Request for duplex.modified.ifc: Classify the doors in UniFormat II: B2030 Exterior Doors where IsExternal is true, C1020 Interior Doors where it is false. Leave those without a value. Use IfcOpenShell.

First a look at what the model holds.

```python
import ifcopenshell
import ifcopenshell.util.element

model = ifcopenshell.open("duplex.modified.ifc")
print(model.schema)
print("classifications:", [c.Name for c in model.by_type("IfcClassification")])
values = [ifcopenshell.util.element.get_pset(e, "Pset_DoorCommon", "IsExternal") for e in model.by_type("IfcDoor")]
for value in (True, False, None):
    print("IsExternal", value, values.count(value))
```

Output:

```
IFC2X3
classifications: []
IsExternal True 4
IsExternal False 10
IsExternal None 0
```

```python
import ifcopenshell
import ifcopenshell.api.classification
import ifcopenshell.util.element

model = ifcopenshell.open("duplex.modified.ifc")

# IFC2X3 requires Source and Edition and has no link from the project to the system.
system = model.create_entity("IfcClassification", Source="ASTM", Edition="E1557", Name="UniFormat II")

doors = model.by_type("IfcDoor")
external = {e: ifcopenshell.util.element.get_pset(e, "Pset_DoorCommon", "IsExternal") for e in doors}
for flag, code, name in ((True, "B2030", "Exterior Doors"), (False, "C1020", "Interior Doors")):
    products = [e for e in doors if external[e] is flag]
    ifcopenshell.api.classification.add_reference(
        model, products=products, classification=system, identification=code, name=name
    )
    print(code, len(products))

model.write("duplex.modified_v2.ifc")
```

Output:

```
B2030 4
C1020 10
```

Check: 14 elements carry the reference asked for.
